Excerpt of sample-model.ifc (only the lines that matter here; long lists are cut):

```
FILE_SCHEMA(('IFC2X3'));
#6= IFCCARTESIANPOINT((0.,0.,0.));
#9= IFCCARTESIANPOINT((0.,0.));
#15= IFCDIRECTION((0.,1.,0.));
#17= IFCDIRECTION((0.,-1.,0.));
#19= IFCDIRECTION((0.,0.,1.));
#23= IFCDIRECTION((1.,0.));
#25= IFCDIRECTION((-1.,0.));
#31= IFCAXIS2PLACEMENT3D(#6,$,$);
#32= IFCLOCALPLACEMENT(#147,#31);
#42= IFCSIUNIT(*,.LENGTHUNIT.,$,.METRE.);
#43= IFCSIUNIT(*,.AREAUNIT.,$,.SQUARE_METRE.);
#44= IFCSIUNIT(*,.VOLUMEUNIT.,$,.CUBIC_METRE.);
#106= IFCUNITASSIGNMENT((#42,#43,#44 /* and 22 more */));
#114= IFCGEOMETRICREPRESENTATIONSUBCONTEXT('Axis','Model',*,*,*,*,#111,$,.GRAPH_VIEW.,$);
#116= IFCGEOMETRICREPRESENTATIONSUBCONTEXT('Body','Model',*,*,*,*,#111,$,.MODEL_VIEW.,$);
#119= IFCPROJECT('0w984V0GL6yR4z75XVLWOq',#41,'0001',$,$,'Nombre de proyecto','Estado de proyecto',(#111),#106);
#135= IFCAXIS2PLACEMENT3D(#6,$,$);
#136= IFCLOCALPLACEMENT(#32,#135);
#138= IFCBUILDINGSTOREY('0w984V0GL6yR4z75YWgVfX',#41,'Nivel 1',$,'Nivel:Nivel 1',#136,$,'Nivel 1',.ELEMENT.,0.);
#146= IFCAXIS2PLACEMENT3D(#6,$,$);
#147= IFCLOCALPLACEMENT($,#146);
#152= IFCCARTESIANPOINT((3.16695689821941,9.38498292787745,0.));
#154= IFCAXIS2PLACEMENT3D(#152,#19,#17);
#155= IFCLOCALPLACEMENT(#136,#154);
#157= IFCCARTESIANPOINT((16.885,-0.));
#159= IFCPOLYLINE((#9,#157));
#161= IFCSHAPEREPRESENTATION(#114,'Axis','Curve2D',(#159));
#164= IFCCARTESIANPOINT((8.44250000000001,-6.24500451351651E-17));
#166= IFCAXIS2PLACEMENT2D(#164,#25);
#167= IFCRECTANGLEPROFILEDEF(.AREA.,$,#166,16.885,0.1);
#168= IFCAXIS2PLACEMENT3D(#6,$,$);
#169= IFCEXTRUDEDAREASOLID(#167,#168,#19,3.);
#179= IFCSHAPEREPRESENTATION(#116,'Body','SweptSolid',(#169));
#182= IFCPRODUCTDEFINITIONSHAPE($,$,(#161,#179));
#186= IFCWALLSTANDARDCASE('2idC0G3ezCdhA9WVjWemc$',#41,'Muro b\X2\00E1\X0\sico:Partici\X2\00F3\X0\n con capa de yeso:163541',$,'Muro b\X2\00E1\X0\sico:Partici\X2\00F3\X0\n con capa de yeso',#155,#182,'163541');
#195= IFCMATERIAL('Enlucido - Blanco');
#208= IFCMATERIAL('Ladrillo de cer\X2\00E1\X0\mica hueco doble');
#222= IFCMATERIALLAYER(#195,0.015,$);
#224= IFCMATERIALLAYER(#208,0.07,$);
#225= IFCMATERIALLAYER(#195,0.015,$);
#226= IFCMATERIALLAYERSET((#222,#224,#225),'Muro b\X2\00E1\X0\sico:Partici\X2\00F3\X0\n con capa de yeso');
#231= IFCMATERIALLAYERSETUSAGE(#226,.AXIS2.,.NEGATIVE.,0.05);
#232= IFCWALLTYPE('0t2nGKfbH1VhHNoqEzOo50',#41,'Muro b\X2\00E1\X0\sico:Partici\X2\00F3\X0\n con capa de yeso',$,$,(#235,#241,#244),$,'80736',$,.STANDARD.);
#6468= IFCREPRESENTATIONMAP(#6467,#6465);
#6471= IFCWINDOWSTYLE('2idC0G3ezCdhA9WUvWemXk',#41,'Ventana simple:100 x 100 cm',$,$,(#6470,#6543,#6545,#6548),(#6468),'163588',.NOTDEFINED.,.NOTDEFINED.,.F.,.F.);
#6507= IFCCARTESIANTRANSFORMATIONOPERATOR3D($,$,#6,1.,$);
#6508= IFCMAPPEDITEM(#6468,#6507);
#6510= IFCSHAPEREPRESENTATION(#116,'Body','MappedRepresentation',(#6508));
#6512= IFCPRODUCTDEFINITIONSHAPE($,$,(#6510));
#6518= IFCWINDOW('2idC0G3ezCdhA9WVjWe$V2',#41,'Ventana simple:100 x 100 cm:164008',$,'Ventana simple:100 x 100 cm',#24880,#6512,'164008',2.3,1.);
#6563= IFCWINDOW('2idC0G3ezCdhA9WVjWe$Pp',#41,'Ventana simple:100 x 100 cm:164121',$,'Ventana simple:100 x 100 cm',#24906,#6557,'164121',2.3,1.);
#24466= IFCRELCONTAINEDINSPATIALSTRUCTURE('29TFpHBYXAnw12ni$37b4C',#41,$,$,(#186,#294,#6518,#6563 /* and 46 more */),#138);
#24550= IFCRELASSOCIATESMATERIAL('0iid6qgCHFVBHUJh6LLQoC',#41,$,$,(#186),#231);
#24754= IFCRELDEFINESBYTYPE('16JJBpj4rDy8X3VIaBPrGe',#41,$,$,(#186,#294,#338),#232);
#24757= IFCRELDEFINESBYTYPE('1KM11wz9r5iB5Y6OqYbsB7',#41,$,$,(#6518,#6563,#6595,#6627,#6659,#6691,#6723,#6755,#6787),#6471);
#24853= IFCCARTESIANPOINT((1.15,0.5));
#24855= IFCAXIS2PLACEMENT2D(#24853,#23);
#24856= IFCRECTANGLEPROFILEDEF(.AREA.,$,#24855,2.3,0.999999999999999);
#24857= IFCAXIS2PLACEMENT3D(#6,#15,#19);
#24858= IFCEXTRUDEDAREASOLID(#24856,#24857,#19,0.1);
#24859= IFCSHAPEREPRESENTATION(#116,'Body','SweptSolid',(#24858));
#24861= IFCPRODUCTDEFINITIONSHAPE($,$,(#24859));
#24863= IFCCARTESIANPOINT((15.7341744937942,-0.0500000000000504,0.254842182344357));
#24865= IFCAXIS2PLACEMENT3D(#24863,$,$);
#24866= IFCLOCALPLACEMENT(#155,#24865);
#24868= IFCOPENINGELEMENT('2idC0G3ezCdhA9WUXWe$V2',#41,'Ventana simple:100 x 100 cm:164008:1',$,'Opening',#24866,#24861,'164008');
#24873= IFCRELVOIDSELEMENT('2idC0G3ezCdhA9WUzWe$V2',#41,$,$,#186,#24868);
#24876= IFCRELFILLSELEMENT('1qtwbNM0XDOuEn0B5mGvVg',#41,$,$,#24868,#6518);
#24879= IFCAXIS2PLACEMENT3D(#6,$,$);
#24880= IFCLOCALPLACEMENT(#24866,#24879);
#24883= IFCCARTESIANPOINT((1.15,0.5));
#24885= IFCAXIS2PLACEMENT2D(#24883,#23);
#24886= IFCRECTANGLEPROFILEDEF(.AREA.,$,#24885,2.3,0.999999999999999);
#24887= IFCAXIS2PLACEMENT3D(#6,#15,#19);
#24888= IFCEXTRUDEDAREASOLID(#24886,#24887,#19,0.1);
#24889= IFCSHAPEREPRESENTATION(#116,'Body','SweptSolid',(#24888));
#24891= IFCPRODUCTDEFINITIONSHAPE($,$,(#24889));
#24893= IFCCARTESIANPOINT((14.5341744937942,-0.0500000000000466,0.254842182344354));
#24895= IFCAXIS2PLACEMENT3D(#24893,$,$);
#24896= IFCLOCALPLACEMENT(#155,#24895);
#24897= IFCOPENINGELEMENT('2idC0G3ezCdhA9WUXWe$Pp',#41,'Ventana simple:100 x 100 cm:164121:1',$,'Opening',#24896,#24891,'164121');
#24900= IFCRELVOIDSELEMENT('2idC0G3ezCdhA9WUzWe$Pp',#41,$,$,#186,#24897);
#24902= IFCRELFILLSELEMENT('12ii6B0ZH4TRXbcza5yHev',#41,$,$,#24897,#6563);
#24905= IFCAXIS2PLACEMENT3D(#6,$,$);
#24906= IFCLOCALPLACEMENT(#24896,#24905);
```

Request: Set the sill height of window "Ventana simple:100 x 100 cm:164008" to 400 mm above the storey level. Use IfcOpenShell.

```python
import numpy as np
import ifcopenshell
import ifcopenshell.api.geometry
import ifcopenshell.geom
import ifcopenshell.util.element
import ifcopenshell.util.placement
import ifcopenshell.util.shape
import ifcopenshell.util.unit

model = ifcopenshell.open("sample-model.ifc")
unit_scale = ifcopenshell.util.unit.calculate_unit_scale(model)

window = model.by_guid("2idC0G3ezCdhA9WVjWe$V2")
opening = window.FillsVoids[0].RelatingOpeningElement
storey = ifcopenshell.util.element.get_container(window, ifc_class="IfcBuildingStorey")
level = ifcopenshell.util.placement.get_local_placement(storey.ObjectPlacement)[2, 3]

# The opening's origin need not be at the sill, so measure its lowest point.
shape = ifcopenshell.geom.create_shape(ifcopenshell.geom.settings(), opening)
bottom = ifcopenshell.util.shape.get_shape_bottom_elevation(shape, shape.geometry) / unit_scale
dz = level + 0.4 / unit_scale - bottom

shift = np.array([0.0, 0.0, dz])
# The window is placed relative to its opening, so it follows when the opening moves.
matrix = ifcopenshell.util.placement.get_local_placement(opening.ObjectPlacement)
matrix[:3, 3] += shift
ifcopenshell.api.geometry.edit_object_placement(
    model, product=opening, matrix=matrix, is_si=False, should_transform_children=True
)

print(f"moved by {dz * unit_scale:+.3f} m")

model.write("sample-model-out.ifc")
```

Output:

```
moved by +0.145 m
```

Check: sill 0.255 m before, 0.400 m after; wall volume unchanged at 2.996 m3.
